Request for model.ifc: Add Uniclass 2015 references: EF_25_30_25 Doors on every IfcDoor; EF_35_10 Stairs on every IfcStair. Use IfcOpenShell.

First a look at what the model holds.

```python
import ifcopenshell

model = ifcopenshell.open("model.ifc")
print(model.schema)
print("classifications:", [c.Name for c in model.by_type("IfcClassification")])
for ifc_class in ("IfcDoor", "IfcRoof", "IfcStair", "IfcWall", "IfcWindow"):
    print(ifc_class, len(model.by_type(ifc_class)))
```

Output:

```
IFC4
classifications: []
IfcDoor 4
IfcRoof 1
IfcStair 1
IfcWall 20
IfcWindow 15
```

```python
import ifcopenshell
import ifcopenshell.api.classification

model = ifcopenshell.open("model.ifc")

system = ifcopenshell.api.classification.add_classification(model, classification="Uniclass 2015")

codes = {
    "IfcDoor": ("EF_25_30_25", "Doors"),
    "IfcStair": ("EF_35_10", "Stairs"),
}
for ifc_class, (code, name) in codes.items():
    products = model.by_type(ifc_class)
    ifcopenshell.api.classification.add_reference(
        model, products=products, classification=system, identification=code, name=name
    )
    print(code, len(products))

model.write("model_rev.ifc")
```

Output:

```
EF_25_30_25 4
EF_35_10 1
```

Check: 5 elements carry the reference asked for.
